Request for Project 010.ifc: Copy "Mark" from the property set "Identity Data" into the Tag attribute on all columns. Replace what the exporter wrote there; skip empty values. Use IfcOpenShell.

First a look at what the model holds.

```python
import ifcopenshell
import ifcopenshell.util.element

model = ifcopenshell.open("Project 010.ifc")
print(model.schema)
columns = model.by_type("IfcColumn")
print(len(columns), "columns")
for e in columns[:8]:
    source = ifcopenshell.util.element.get_pset(e, "Identity Data", "Mark")
    target = e.Tag
    print(e.id(), repr(source), repr(target), sep=" | ")
```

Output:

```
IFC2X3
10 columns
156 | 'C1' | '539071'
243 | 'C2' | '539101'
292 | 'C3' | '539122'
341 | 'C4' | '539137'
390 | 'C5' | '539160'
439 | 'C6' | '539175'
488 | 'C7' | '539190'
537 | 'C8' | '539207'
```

```python
import ifcopenshell
import ifcopenshell.util.element

model = ifcopenshell.open("Project 010.ifc")

count = 0
for e in model.by_type("IfcColumn"):
    value = ifcopenshell.util.element.get_pset(e, "Identity Data", "Mark")
    current = e.Tag
    if not value or not value.strip() or current == value:
        continue
    e.Tag = value
    count += 1

print(count, "columns updated")

model.write("Project 010_rev.ifc")
```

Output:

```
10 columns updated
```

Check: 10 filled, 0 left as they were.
